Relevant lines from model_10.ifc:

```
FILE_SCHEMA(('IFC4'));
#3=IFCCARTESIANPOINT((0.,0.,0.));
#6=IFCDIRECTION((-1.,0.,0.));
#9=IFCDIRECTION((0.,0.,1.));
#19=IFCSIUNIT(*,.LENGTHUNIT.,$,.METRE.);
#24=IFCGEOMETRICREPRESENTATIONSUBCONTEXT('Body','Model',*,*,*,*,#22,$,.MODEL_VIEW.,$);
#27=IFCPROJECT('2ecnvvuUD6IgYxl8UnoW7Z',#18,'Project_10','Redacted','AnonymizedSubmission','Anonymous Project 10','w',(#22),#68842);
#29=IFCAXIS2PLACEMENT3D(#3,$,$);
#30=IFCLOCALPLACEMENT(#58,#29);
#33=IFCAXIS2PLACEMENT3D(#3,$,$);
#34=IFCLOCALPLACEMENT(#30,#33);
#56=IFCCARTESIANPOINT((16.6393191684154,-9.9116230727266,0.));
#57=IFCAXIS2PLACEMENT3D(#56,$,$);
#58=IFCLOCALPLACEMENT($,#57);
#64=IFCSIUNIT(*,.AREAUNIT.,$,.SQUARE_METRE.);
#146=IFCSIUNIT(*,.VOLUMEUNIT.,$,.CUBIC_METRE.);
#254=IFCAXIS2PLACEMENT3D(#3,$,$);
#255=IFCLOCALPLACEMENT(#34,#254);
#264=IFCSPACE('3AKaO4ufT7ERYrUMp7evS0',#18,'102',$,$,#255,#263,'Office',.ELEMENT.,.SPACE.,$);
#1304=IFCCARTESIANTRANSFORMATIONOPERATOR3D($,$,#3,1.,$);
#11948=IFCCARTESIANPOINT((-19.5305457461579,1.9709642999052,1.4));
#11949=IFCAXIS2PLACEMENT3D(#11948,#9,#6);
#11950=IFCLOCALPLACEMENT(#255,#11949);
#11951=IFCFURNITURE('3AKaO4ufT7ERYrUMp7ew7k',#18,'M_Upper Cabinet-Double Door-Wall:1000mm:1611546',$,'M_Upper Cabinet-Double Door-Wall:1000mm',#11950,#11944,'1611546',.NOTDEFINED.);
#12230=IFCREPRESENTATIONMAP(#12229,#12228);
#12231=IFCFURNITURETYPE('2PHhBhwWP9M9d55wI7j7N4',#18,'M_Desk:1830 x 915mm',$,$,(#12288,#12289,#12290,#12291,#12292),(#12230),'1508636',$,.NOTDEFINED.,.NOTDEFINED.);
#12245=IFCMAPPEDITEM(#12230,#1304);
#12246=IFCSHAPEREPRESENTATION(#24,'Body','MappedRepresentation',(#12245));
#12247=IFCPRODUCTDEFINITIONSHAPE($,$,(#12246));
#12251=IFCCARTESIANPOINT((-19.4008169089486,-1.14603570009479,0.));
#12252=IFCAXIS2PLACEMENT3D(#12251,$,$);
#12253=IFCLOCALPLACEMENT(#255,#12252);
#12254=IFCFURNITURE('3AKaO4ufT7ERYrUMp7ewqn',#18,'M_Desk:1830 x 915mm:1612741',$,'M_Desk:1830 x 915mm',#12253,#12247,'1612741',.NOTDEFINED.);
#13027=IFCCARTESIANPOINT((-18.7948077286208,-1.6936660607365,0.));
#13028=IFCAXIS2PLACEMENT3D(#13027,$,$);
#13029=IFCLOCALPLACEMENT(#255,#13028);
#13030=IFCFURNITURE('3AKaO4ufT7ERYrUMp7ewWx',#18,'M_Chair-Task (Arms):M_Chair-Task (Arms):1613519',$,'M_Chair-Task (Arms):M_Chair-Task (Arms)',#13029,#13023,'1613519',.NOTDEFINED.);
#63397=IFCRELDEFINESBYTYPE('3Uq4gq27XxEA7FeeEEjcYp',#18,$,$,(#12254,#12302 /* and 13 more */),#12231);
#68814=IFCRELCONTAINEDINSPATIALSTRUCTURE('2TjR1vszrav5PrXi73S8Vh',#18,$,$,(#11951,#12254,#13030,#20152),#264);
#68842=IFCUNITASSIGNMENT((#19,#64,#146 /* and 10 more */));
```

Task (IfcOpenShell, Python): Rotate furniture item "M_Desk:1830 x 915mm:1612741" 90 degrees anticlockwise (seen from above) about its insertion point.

```python
import ifcopenshell
import ifcopenshell.api.geometry
import ifcopenshell.util.placement

model = ifcopenshell.open("model_10.ifc")

item = model.by_id(12254)
matrix = ifcopenshell.util.placement.get_local_placement(item.ObjectPlacement)
matrix = matrix @ ifcopenshell.util.placement.rotation(90, "Z")
ifcopenshell.api.geometry.edit_object_placement(model, product=item, matrix=matrix, is_si=False)

print(ifcopenshell.util.placement.get_local_placement(item.ObjectPlacement).round(3) + 0.0)

model.write("model_10_rev.ifc")
```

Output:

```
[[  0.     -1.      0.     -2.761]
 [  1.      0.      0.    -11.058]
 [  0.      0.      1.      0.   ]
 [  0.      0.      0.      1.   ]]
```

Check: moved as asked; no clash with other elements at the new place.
